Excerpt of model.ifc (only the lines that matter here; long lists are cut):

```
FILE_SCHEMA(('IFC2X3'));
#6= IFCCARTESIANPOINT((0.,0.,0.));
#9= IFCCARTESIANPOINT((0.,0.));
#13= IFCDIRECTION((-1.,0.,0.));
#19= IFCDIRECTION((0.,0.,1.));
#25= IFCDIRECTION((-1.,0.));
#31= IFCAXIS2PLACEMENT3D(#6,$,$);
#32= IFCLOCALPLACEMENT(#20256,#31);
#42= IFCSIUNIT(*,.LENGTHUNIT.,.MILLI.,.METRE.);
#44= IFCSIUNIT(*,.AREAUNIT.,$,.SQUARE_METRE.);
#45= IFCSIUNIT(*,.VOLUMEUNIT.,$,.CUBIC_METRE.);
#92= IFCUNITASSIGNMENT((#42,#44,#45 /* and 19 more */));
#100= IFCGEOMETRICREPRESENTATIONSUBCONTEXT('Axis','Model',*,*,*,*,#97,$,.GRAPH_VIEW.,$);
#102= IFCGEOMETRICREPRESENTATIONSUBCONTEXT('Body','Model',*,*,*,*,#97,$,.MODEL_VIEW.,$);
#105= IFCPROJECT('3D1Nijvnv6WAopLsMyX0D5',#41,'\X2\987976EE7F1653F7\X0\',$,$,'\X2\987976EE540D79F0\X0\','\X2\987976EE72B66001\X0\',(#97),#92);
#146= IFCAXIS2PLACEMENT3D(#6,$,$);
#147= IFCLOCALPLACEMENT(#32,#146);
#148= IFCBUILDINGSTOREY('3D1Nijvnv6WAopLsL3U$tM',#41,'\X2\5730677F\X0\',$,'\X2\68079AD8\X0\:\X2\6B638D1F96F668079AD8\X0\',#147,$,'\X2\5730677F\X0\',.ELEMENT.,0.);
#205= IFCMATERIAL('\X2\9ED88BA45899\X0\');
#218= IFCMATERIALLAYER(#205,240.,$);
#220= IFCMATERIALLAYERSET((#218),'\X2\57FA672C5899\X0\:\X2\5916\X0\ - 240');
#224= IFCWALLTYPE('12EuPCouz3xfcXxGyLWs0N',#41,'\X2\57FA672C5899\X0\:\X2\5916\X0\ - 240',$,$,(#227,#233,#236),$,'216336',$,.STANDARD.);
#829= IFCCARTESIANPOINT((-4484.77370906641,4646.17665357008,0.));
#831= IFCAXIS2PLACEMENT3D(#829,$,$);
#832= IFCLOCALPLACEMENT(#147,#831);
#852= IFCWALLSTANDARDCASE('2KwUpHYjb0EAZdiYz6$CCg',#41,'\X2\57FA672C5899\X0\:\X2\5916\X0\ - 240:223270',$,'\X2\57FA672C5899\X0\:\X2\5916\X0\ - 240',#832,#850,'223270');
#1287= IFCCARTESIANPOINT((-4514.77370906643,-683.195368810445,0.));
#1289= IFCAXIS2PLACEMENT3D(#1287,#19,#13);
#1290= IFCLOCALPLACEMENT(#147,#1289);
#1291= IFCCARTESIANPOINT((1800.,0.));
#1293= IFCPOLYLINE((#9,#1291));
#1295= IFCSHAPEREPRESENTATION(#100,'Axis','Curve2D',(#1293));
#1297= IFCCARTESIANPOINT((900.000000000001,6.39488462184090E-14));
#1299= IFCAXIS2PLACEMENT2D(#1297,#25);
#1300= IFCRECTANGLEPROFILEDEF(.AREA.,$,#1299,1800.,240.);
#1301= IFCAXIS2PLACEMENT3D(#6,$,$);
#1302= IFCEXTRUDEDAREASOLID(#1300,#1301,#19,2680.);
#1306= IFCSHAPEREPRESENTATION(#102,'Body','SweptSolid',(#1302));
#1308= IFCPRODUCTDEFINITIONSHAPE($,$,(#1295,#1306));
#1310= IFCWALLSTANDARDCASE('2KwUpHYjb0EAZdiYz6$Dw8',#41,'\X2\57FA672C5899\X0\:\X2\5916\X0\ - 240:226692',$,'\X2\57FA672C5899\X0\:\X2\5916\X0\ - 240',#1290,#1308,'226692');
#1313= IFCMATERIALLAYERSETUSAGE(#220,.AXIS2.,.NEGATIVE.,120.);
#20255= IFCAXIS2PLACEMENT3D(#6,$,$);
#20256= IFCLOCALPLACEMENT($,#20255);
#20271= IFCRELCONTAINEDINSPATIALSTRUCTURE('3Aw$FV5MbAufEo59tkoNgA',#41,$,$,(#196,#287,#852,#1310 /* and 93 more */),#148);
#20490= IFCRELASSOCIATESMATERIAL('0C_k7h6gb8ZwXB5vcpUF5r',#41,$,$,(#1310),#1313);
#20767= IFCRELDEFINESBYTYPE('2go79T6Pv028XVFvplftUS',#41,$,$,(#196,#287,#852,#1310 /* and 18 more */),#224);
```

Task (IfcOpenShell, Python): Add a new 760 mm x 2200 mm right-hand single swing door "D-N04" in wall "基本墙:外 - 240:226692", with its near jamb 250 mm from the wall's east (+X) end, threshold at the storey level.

```python
import numpy as np
import ifcopenshell
import ifcopenshell.api.feature
import ifcopenshell.api.geometry
import ifcopenshell.api.root
import ifcopenshell.api.spatial
import ifcopenshell.api.type
import ifcopenshell.geom
import ifcopenshell.util.element
import ifcopenshell.util.placement
import ifcopenshell.util.representation
import ifcopenshell.util.shape
import ifcopenshell.util.unit

model = ifcopenshell.open("model.ifc")
unit_scale = ifcopenshell.util.unit.calculate_unit_scale(model)
settings = ifcopenshell.geom.settings()


def volume(element):
    """Net volume in cubic metres, openings subtracted."""
    shape = ifcopenshell.geom.create_shape(settings, element)
    return ifcopenshell.util.shape.get_volume(shape.geometry)


wall = model.by_guid("2KwUpHYjb0EAZdiYz6$Dw8")
storey = ifcopenshell.util.element.get_container(wall, ifc_class="IfcBuildingStorey")
context = ifcopenshell.util.representation.get_context(model, "Model", "Body", "MODEL_VIEW")
before = volume(wall)

width, height, from_end, sill = 0.76, 2.2, 0.25, 0.0  # metres

# The wall runs along its own X axis, and the end named is its -X end.
wall_shape = ifcopenshell.geom.create_shape(settings, wall)
x, y, z = ifcopenshell.util.shape.get_vertices(wall_shape.geometry).T
start = x.min() + from_end
face, thickness = float(y.min()), float(y.max() - y.min())
wall_matrix = ifcopenshell.util.placement.get_local_placement(wall.ObjectPlacement)
level = ifcopenshell.util.placement.get_local_placement(storey.ObjectPlacement)[2, 3]


def in_wall(x, y):
    """Placement at x, y metres in the wall's axes, at sill height."""
    matrix = wall_matrix.copy()
    matrix[:, 3] = wall_matrix @ np.array([x / unit_scale, y / unit_scale, 0.0, 1.0])
    matrix[2, 3] = level + sill / unit_scale
    return matrix


# Opening: a box that overshoots both wall faces by 50 mm.
opening = ifcopenshell.api.root.create_entity(model, ifc_class="IfcOpeningElement")
box = ifcopenshell.api.geometry.add_wall_representation(
    model, context=context, length=width, height=height, thickness=thickness + 0.1
)
ifcopenshell.api.geometry.assign_representation(model, product=opening, representation=box)
ifcopenshell.api.geometry.edit_object_placement(model, product=opening, matrix=in_wall(start, face - 0.05), is_si=False)
ifcopenshell.api.feature.add_feature(model, feature=opening, element=wall)

door = ifcopenshell.api.root.create_entity(model, ifc_class="IfcDoor", name="D-N04")
door.OverallWidth, door.OverallHeight = width / unit_scale, height / unit_scale
body = ifcopenshell.api.geometry.add_door_representation(
    model,
    context=context,
    overall_width=door.OverallWidth,
    overall_height=door.OverallHeight,
    operation_type="SINGLE_SWING_RIGHT",
    lining_properties={"LiningDepth": thickness / unit_scale, "ThresholdDepth": thickness / unit_scale},
)
ifcopenshell.api.geometry.assign_representation(model, product=door, representation=body)
ifcopenshell.api.spatial.assign_container(model, products=[door], relating_structure=storey)
fills = ifcopenshell.api.feature.add_filling(model, opening=opening, element=door)
fills.OwnerHistory = door.OwnerHistory  # required in IFC2X3

# IFC2X3 keeps the operation on the door style.
style = ifcopenshell.api.root.create_entity(model, ifc_class="IfcDoorStyle", name="D-N04")
style.OperationType, style.ConstructionType = "SINGLE_SWING_RIGHT", "NOTDEFINED"
style.ParameterTakesPrecedence = style.Sizeable = False
ifcopenshell.api.type.assign_type(model, related_objects=[door], relating_type=style)

# The lining spans the wall, so the door starts at the wall face.
ifcopenshell.api.geometry.edit_object_placement(model, product=door, matrix=in_wall(start, face), is_si=False)

after = volume(wall)

print(f"wall volume {before:.3f} -> {after:.3f} m3")

model.write("model_updated.ifc")
```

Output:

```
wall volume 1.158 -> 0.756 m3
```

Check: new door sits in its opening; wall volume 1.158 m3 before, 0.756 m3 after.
